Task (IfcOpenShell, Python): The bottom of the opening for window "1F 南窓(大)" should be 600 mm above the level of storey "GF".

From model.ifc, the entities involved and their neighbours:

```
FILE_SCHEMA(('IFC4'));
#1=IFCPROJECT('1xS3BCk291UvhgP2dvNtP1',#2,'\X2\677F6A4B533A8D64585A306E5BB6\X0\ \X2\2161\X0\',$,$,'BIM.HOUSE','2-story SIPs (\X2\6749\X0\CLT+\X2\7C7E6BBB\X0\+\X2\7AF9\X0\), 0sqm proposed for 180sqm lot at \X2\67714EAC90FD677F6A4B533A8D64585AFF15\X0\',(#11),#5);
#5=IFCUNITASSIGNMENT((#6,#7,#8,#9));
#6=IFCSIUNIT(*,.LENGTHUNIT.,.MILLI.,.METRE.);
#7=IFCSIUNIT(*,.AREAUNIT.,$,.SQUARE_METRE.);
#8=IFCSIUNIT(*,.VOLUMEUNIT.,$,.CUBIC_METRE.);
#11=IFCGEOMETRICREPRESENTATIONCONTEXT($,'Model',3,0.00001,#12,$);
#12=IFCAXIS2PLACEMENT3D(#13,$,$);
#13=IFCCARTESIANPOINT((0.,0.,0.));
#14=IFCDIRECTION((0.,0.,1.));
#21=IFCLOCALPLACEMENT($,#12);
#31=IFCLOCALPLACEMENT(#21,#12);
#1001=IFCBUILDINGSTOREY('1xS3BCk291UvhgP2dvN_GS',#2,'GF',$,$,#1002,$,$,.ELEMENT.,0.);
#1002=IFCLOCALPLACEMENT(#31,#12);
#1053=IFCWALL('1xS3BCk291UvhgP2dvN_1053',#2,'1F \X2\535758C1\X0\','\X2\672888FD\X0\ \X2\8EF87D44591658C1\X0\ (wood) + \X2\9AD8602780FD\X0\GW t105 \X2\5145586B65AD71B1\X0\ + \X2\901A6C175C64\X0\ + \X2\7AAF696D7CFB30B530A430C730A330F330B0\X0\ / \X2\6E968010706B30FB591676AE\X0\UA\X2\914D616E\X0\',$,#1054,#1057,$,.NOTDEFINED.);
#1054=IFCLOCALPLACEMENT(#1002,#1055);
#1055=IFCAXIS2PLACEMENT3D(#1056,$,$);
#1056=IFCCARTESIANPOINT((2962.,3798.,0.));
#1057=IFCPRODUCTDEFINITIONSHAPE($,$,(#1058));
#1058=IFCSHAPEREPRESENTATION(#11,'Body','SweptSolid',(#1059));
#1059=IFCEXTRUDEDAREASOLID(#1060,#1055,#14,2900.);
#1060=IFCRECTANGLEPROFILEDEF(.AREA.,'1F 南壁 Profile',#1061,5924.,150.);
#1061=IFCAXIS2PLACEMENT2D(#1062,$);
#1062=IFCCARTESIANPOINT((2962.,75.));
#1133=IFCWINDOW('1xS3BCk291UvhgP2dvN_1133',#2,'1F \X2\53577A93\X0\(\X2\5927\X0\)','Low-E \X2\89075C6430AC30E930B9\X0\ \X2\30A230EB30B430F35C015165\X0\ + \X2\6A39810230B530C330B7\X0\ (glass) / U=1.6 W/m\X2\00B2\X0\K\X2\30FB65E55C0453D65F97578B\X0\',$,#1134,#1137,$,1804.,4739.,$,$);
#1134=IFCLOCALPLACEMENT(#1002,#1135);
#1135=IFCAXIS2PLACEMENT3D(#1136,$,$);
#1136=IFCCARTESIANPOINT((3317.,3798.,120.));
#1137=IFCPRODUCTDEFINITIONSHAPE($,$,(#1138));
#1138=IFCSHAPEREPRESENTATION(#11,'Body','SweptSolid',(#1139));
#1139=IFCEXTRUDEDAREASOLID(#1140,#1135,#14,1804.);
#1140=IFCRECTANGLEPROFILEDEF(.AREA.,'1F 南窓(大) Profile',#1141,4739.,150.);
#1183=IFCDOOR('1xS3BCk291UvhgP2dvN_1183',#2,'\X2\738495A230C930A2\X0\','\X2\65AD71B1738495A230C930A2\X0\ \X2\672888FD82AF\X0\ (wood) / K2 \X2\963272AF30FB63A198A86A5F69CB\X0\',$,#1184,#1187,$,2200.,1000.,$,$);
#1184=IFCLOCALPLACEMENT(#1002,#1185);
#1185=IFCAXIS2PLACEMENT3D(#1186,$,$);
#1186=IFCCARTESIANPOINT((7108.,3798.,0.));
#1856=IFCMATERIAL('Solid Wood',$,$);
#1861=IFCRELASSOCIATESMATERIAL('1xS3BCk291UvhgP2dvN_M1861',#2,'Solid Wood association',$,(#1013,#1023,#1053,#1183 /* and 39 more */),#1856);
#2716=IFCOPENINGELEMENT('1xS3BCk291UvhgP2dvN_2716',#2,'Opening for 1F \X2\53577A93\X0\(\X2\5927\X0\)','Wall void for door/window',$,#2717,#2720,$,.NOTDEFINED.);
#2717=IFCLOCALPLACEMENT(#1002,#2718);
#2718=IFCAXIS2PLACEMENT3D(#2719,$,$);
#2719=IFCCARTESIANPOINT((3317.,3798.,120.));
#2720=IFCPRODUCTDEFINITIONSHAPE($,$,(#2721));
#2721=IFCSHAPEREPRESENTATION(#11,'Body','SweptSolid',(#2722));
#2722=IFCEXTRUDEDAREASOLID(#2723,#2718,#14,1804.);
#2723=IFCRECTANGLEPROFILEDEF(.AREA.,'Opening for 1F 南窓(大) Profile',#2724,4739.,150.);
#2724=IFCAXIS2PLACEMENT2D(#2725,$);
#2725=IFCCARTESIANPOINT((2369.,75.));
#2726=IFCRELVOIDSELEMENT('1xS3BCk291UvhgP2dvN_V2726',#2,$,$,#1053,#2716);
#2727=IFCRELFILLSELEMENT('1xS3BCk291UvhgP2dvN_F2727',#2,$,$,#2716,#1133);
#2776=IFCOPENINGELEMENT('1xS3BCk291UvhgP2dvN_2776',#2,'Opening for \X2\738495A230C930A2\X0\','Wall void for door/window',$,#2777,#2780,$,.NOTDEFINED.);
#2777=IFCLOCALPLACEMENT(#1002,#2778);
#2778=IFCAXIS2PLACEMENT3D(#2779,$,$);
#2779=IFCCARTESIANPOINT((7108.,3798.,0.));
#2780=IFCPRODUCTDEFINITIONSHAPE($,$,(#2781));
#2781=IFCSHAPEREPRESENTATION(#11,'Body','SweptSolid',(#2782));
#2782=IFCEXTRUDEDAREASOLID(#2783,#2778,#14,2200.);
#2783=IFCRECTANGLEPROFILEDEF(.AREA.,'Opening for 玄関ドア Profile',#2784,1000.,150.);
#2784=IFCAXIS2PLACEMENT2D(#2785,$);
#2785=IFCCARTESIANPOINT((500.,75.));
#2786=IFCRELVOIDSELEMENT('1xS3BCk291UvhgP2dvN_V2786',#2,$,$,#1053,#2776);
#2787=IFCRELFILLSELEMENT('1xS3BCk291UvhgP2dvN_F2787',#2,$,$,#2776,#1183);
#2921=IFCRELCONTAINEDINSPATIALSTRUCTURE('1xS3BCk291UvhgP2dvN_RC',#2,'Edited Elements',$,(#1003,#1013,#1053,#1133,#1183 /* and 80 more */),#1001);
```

```python
import numpy as np
import ifcopenshell
import ifcopenshell.api.geometry
import ifcopenshell.geom
import ifcopenshell.util.element
import ifcopenshell.util.placement
import ifcopenshell.util.shape
import ifcopenshell.util.unit

model = ifcopenshell.open("model.ifc")
unit_scale = ifcopenshell.util.unit.calculate_unit_scale(model)

window = model.by_guid("1xS3BCk291UvhgP2dvN_1133")
opening = window.FillsVoids[0].RelatingOpeningElement
storey = ifcopenshell.util.element.get_container(window, ifc_class="IfcBuildingStorey")
level = ifcopenshell.util.placement.get_local_placement(storey.ObjectPlacement)[2, 3]

# The opening's origin need not be at the sill, so measure its lowest point.
shape = ifcopenshell.geom.create_shape(ifcopenshell.geom.settings(), opening)
bottom = ifcopenshell.util.shape.get_shape_bottom_elevation(shape, shape.geometry) / unit_scale
dz = level + 600.0 - bottom

shift = np.array([0.0, 0.0, dz])
# The window is not placed relative to its opening, so move both.
for product in (opening, window):
    matrix = ifcopenshell.util.placement.get_local_placement(product.ObjectPlacement)
    matrix[:3, 3] += shift
    ifcopenshell.api.geometry.edit_object_placement(model, product=product, matrix=matrix, is_si=False)

print(f"moved by {dz * unit_scale:+.3f} m")

model.write("model_updated.ifc")
```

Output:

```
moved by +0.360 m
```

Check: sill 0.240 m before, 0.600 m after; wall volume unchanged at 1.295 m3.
